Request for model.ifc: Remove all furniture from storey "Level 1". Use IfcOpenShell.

First a look at what the model holds.

```python
import ifcopenshell
import ifcopenshell.util.element

model = ifcopenshell.open("model.ifc")
print(model.schema)
storey = next(s for s in model.by_type("IfcBuildingStorey") if s.Name == "Level 1")
furniture = [e for e in ifcopenshell.util.element.get_decomposition(storey) if e.is_a("IfcFurnishingElement")]
seen = {}
for e in furniture:
    element_type = ifcopenshell.util.element.get_type(e)
    name = element_type.Name if element_type not in (None, e) else None
    seen[name] = seen.get(name, 0) + 1
for name, count in sorted(seen.items(), key=str):
    print(count, "x", name)
```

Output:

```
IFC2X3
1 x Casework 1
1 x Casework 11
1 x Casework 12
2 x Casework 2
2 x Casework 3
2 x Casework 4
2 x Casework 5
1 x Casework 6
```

```python
import ifcopenshell
import ifcopenshell.api.root
import ifcopenshell.util.element

model = ifcopenshell.open("model.ifc")

storey = next(s for s in model.by_type("IfcBuildingStorey") if s.Name == "Level 1")
furniture = [e for e in ifcopenshell.util.element.get_decomposition(storey) if e.is_a("IfcFurnishingElement")]

for e in furniture:
    ifcopenshell.api.root.remove_product(model, product=e)
print(len(furniture), "removed")

model.write("model_v2.ifc")
```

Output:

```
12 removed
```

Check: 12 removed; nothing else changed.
